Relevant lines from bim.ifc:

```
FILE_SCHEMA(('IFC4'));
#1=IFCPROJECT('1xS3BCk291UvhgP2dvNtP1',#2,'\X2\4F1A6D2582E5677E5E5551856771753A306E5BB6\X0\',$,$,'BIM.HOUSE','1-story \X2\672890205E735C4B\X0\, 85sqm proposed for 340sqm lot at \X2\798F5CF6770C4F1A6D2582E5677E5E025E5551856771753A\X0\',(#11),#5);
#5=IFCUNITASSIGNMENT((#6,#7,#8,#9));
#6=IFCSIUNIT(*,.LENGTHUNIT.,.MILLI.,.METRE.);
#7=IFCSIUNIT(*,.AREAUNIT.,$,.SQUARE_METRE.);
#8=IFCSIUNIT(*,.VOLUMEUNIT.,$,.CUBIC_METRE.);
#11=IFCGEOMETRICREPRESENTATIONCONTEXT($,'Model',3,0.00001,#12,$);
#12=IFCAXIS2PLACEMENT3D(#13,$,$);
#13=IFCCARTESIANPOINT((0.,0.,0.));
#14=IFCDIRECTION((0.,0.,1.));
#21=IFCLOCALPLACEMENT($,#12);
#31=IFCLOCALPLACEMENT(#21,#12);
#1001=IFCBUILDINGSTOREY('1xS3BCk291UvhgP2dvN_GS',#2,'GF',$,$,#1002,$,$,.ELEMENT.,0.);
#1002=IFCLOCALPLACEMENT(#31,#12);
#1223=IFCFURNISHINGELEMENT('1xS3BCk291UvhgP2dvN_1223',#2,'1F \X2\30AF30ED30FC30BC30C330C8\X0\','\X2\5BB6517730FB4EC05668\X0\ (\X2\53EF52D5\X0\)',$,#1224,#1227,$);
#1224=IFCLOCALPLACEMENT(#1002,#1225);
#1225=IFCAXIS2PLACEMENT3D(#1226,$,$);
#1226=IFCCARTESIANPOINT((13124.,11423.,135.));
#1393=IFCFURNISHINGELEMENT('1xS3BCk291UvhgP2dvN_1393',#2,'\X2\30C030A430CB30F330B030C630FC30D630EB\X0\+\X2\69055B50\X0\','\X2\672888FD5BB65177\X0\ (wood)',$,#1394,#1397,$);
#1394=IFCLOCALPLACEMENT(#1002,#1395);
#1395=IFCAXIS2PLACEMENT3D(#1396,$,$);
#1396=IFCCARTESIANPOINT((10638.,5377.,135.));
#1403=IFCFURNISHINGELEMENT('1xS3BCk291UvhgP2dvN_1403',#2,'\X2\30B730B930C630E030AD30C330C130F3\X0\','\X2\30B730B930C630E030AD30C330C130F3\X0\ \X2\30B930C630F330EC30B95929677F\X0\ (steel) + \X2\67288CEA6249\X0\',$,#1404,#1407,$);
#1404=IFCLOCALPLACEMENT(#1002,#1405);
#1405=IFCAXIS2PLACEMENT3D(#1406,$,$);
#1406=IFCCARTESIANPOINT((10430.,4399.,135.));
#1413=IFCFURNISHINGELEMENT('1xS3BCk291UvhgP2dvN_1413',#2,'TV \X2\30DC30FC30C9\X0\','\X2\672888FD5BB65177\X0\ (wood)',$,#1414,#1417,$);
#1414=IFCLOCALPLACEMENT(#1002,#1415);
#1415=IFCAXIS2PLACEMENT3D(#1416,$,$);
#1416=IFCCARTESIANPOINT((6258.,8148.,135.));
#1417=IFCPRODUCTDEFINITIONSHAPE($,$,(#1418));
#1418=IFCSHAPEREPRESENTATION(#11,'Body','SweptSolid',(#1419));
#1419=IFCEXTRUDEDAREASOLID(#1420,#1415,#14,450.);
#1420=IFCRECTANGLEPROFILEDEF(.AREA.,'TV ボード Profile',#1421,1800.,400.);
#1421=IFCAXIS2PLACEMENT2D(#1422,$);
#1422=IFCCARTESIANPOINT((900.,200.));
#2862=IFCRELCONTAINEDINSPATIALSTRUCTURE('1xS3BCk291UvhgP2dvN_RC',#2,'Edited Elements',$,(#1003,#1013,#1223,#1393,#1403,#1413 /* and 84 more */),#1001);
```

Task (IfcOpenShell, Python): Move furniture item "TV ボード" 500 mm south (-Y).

```python
import ifcopenshell
import ifcopenshell.api.geometry
import ifcopenshell.util.placement

model = ifcopenshell.open("bim.ifc")

item = model.by_guid("1xS3BCk291UvhgP2dvN_1413")
matrix = ifcopenshell.util.placement.get_local_placement(item.ObjectPlacement)
matrix[1, 3] -= 500.0
ifcopenshell.api.geometry.edit_object_placement(model, product=item, matrix=matrix, is_si=False)

print(ifcopenshell.util.placement.get_local_placement(item.ObjectPlacement).round(3) + 0.0)

model.write("bim_v2.ifc")
```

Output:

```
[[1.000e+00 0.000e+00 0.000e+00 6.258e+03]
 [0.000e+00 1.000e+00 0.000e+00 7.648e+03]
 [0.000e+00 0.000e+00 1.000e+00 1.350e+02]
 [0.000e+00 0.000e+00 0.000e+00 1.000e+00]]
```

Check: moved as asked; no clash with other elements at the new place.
